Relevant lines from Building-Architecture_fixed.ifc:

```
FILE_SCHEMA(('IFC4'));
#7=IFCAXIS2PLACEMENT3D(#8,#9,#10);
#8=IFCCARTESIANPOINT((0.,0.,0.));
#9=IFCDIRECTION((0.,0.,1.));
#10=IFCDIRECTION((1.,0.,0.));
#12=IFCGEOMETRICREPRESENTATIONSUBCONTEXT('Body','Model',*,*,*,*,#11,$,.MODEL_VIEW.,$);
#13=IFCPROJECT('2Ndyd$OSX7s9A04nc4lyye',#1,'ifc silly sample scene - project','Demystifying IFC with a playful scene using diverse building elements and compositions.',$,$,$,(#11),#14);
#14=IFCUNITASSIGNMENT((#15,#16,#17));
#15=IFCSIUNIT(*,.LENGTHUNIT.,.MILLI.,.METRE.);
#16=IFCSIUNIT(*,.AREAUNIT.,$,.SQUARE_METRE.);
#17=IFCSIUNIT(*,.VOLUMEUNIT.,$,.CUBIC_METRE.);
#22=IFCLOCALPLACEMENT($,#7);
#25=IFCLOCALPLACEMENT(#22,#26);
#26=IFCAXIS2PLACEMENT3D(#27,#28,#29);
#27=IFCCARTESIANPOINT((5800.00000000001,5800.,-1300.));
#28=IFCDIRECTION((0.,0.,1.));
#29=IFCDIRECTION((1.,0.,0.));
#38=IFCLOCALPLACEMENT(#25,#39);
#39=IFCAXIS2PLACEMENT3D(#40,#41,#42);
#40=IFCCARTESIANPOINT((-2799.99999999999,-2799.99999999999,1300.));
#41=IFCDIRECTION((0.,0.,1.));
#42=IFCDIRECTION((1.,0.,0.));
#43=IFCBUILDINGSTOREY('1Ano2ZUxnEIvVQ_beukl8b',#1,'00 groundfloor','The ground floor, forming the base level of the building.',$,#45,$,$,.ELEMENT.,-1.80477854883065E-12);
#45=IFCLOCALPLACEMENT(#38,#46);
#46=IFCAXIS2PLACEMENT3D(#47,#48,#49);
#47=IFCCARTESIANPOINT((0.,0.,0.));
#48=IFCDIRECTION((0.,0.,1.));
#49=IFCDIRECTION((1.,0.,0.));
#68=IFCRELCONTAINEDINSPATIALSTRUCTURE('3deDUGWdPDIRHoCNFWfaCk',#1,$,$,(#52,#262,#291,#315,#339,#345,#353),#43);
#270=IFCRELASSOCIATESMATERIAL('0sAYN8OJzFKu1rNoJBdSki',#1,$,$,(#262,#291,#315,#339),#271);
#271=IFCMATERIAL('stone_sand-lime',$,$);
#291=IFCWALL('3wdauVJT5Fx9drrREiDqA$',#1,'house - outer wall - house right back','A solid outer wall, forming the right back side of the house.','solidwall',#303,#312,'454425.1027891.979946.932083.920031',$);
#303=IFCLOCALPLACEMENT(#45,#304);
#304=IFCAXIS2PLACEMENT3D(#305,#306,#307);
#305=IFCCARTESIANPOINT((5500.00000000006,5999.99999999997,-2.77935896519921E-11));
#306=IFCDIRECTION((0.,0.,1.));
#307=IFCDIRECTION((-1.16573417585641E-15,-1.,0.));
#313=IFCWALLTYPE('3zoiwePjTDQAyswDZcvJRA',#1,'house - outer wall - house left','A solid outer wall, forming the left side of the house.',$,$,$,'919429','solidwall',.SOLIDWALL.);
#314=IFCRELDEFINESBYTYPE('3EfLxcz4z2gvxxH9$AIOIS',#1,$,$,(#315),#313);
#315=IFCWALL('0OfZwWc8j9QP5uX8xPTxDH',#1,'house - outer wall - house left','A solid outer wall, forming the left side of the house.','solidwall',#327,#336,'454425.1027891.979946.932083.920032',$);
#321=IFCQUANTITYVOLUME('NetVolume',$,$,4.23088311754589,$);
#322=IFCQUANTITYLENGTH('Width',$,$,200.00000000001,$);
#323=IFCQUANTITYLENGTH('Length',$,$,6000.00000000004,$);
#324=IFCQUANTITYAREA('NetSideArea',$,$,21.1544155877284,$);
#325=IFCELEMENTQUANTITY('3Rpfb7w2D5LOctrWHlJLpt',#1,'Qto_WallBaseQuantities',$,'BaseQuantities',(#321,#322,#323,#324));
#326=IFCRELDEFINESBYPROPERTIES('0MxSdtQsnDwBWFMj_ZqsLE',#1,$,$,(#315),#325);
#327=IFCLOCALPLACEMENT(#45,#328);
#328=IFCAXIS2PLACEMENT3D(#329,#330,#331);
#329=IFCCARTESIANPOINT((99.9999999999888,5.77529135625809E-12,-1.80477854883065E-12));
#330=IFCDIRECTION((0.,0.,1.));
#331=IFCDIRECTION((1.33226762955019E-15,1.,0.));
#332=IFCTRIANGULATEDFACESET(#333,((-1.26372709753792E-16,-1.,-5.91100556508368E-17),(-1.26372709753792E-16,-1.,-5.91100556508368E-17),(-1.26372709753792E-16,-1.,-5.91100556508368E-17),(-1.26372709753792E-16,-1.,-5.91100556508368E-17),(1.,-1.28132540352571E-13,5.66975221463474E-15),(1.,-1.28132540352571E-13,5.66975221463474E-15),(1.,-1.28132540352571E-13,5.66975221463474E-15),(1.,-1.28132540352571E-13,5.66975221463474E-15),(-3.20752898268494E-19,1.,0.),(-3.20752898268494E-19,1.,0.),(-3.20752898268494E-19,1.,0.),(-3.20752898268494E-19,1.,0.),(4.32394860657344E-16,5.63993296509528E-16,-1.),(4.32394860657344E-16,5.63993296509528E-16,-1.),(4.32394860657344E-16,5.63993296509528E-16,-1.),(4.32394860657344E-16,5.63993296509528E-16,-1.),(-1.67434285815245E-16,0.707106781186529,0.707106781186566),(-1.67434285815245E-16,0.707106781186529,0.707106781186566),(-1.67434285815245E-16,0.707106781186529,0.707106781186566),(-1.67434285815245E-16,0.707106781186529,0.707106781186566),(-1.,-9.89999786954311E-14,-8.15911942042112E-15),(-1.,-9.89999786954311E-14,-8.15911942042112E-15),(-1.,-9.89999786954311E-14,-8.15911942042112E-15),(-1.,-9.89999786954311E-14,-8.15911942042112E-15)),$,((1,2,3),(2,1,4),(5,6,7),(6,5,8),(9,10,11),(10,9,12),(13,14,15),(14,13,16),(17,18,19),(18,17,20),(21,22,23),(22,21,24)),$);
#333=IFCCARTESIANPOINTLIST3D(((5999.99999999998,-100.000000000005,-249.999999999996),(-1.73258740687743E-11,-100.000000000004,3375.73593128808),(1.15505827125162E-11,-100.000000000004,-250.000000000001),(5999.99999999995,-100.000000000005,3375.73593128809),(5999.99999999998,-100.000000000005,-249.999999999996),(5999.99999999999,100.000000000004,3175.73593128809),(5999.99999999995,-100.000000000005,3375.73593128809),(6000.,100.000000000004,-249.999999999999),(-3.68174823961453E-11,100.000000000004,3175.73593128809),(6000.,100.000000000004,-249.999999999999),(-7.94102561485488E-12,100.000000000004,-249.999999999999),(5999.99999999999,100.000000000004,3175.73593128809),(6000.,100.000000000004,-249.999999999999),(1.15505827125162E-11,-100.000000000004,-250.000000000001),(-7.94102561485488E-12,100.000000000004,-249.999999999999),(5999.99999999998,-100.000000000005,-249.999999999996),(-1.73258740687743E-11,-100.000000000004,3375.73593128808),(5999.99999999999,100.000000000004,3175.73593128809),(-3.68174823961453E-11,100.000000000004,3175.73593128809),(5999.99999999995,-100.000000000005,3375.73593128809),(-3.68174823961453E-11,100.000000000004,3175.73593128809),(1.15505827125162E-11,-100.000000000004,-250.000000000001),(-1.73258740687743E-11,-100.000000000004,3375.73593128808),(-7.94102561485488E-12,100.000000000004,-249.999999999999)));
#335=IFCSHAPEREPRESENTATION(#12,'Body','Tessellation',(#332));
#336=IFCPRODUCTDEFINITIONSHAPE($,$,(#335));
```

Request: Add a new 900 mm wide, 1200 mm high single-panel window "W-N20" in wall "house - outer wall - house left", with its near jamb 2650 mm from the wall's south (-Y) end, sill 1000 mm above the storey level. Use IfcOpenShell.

```python
import numpy as np
import ifcopenshell
import ifcopenshell.api.feature
import ifcopenshell.api.geometry
import ifcopenshell.api.pset
import ifcopenshell.api.root
import ifcopenshell.api.spatial
import ifcopenshell.geom
import ifcopenshell.util.element
import ifcopenshell.util.placement
import ifcopenshell.util.representation
import ifcopenshell.util.shape
import ifcopenshell.util.unit

model = ifcopenshell.open("Building-Architecture_fixed.ifc")
unit_scale = ifcopenshell.util.unit.calculate_unit_scale(model)
area_scale = ifcopenshell.util.unit.calculate_unit_scale(model, "AREAUNIT")
volume_scale = ifcopenshell.util.unit.calculate_unit_scale(model, "VOLUMEUNIT")
settings = ifcopenshell.geom.settings()


def volume(element):
    """Net volume in cubic metres, openings subtracted."""
    shape = ifcopenshell.geom.create_shape(settings, element)
    return ifcopenshell.util.shape.get_volume(shape.geometry)


wall = model.by_guid("0OfZwWc8j9QP5uX8xPTxDH")
storey = ifcopenshell.util.element.get_container(wall, ifc_class="IfcBuildingStorey")
context = ifcopenshell.util.representation.get_context(model, "Model", "Body", "MODEL_VIEW")
before = volume(wall)

width, height, from_end, sill = 0.9, 1.2, 2.65, 1  # metres

# The wall runs along its own X axis, and the end named is its -X end.
wall_shape = ifcopenshell.geom.create_shape(settings, wall)
x, y, z = ifcopenshell.util.shape.get_vertices(wall_shape.geometry).T
start = x.min() + from_end
face, thickness = float(y.min()), float(y.max() - y.min())
wall_matrix = ifcopenshell.util.placement.get_local_placement(wall.ObjectPlacement)
level = ifcopenshell.util.placement.get_local_placement(storey.ObjectPlacement)[2, 3]


def in_wall(x, y):
    """Placement at x, y metres in the wall's axes, at sill height."""
    matrix = wall_matrix.copy()
    matrix[:, 3] = wall_matrix @ np.array([x / unit_scale, y / unit_scale, 0.0, 1.0])
    matrix[2, 3] = level + sill / unit_scale
    return matrix


# Opening: a box that overshoots both wall faces by 50 mm.
opening = ifcopenshell.api.root.create_entity(model, ifc_class="IfcOpeningElement", predefined_type="OPENING")
box = ifcopenshell.api.geometry.add_wall_representation(
    model, context=context, length=width, height=height, thickness=thickness + 0.1
)
ifcopenshell.api.geometry.assign_representation(model, product=opening, representation=box)
ifcopenshell.api.geometry.edit_object_placement(model, product=opening, matrix=in_wall(start, face - 0.05), is_si=False)
ifcopenshell.api.feature.add_feature(model, feature=opening, element=wall)

window = ifcopenshell.api.root.create_entity(model, ifc_class="IfcWindow", name="W-N20", predefined_type="WINDOW")
window.OverallWidth, window.OverallHeight = width / unit_scale, height / unit_scale
window.PartitioningType = "SINGLE_PANEL"
body = ifcopenshell.api.geometry.add_window_representation(
    model,
    context=context,
    overall_width=window.OverallWidth,
    overall_height=window.OverallHeight,
    partition_type="SINGLE_PANEL",
)
ifcopenshell.api.geometry.assign_representation(model, product=window, representation=body)
ifcopenshell.api.spatial.assign_container(model, products=[window], relating_structure=storey)
ifcopenshell.api.feature.add_filling(model, opening=opening, element=window)

# Centre the window in the wall's thickness.
ifcopenshell.api.geometry.edit_object_placement(model, product=window, matrix=in_wall(start, face), is_si=False)
window_shape = ifcopenshell.geom.create_shape(settings, window)
depth = ifcopenshell.util.shape.get_vertices(window_shape.geometry)[:, 1]
offset = face + thickness / 2 - (depth.min() + depth.max()) / 2
ifcopenshell.api.geometry.edit_object_placement(model, product=window, matrix=in_wall(start, offset), is_si=False)

after = volume(wall)

# Update the wall's stored quantities.
qto = model.by_id(ifcopenshell.util.element.get_pset(wall, "Qto_WallBaseQuantities", should_inherit=False)["id"])
ifcopenshell.api.pset.edit_qto(model, qto=qto, properties={
    "NetVolume": after / volume_scale,
    "NetSideArea": after / thickness / area_scale,
})

print(f"wall volume {before:.3f} -> {after:.3f} m3")

model.write("Building-Architecture_fixed_updated.ifc")
```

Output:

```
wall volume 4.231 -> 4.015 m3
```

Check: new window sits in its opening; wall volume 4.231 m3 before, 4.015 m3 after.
